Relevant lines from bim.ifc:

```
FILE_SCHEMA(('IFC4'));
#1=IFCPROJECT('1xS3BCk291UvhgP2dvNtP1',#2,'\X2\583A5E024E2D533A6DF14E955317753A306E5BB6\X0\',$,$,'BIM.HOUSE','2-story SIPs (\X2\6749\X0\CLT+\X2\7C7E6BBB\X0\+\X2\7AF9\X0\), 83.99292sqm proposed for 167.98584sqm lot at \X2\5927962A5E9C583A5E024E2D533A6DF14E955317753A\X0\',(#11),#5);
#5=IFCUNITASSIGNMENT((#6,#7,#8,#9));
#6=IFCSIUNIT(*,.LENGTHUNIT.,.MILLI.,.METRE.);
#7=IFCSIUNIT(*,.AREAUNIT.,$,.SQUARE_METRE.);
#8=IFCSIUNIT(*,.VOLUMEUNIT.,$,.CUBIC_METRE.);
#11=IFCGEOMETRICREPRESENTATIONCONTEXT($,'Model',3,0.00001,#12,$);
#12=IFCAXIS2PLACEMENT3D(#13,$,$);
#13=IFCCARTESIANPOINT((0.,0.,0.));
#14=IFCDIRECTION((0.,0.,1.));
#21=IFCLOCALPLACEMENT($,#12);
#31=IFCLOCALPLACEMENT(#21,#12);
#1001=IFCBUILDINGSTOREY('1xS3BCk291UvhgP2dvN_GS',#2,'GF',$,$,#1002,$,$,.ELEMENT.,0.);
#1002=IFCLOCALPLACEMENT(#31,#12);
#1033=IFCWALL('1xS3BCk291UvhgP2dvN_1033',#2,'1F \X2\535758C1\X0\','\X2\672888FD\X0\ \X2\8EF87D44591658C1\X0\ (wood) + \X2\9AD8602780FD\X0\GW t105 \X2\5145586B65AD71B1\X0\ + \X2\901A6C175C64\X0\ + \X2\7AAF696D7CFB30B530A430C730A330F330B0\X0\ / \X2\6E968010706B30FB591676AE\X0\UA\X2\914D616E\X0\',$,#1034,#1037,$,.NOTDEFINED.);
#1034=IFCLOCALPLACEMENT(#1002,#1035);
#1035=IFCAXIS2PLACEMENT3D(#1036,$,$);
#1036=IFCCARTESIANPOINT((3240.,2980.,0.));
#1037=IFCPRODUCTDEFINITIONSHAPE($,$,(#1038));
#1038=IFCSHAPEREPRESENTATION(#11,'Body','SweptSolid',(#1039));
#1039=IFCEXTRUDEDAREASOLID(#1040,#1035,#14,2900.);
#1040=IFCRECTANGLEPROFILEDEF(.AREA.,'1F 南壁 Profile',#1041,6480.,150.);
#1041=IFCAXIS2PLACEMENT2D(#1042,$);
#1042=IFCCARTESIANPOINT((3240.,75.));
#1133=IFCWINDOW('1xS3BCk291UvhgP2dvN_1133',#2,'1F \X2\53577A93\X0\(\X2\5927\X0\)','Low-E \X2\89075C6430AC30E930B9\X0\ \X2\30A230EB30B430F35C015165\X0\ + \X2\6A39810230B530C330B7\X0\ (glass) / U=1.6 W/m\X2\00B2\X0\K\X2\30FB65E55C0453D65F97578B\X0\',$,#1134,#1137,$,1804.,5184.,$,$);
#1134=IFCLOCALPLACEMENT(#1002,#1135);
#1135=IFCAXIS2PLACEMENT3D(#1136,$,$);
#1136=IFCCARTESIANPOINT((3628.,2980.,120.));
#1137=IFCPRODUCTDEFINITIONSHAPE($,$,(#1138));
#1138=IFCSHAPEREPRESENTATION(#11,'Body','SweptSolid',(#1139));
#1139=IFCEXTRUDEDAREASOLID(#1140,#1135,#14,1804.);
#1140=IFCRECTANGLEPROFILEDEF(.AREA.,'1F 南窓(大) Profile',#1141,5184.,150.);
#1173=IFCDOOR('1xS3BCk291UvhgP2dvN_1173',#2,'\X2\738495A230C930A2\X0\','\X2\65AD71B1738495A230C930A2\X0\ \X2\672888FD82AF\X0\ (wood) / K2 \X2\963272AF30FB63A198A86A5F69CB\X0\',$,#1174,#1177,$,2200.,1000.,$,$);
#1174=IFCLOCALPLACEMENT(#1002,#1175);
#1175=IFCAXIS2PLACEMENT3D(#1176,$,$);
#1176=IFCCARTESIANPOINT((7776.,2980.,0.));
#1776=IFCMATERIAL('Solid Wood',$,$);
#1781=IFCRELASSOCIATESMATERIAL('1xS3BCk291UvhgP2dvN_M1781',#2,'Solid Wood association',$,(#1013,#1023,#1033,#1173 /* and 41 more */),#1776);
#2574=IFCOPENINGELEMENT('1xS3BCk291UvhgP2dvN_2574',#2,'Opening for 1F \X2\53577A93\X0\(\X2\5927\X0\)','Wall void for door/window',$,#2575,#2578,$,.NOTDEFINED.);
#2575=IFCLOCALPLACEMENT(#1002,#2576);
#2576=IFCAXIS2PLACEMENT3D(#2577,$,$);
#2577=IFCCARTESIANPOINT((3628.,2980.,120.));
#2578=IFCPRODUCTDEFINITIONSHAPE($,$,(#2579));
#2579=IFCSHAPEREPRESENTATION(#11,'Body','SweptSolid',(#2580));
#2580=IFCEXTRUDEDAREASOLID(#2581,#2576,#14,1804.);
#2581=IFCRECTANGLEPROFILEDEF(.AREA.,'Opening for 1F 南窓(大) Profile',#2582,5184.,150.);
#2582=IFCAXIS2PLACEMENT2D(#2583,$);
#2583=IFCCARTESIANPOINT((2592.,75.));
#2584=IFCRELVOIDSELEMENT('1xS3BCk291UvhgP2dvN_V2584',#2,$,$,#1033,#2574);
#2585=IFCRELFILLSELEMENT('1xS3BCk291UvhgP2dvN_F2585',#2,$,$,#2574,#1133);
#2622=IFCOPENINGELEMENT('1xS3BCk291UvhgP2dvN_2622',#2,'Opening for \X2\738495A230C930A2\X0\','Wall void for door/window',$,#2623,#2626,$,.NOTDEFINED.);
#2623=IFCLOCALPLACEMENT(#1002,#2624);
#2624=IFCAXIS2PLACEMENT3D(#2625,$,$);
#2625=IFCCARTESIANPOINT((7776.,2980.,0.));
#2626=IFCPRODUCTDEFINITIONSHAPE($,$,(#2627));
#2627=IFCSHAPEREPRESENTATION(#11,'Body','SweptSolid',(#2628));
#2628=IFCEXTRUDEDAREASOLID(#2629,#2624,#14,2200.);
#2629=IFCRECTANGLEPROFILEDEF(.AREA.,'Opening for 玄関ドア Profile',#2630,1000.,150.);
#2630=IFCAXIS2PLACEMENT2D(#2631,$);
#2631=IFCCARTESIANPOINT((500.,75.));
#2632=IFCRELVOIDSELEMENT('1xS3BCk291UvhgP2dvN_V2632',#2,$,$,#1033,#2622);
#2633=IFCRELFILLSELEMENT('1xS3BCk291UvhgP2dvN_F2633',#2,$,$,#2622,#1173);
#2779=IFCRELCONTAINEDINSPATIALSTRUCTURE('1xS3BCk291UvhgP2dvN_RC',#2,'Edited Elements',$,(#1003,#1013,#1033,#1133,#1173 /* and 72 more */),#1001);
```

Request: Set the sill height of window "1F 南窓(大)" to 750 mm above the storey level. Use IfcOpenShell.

```python
import numpy as np
import ifcopenshell
import ifcopenshell.api.geometry
import ifcopenshell.geom
import ifcopenshell.util.element
import ifcopenshell.util.placement
import ifcopenshell.util.shape
import ifcopenshell.util.unit

model = ifcopenshell.open("bim.ifc")
unit_scale = ifcopenshell.util.unit.calculate_unit_scale(model)

window = model.by_guid("1xS3BCk291UvhgP2dvN_1133")
opening = window.FillsVoids[0].RelatingOpeningElement
storey = ifcopenshell.util.element.get_container(window, ifc_class="IfcBuildingStorey")
level = ifcopenshell.util.placement.get_local_placement(storey.ObjectPlacement)[2, 3]

# The opening's origin need not be at the sill, so measure its lowest point.
shape = ifcopenshell.geom.create_shape(ifcopenshell.geom.settings(), opening)
bottom = ifcopenshell.util.shape.get_shape_bottom_elevation(shape, shape.geometry) / unit_scale
dz = level + 750.0 - bottom

shift = np.array([0.0, 0.0, dz])
# The window is not placed relative to its opening, so move both.
for product in (opening, window):
    matrix = ifcopenshell.util.placement.get_local_placement(product.ObjectPlacement)
    matrix[:3, 3] += shift
    ifcopenshell.api.geometry.edit_object_placement(model, product=product, matrix=matrix, is_si=False)

print(f"moved by {dz * unit_scale:+.3f} m")

model.write("bim-out.ifc")
```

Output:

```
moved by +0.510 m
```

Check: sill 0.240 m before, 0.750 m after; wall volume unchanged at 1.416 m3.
